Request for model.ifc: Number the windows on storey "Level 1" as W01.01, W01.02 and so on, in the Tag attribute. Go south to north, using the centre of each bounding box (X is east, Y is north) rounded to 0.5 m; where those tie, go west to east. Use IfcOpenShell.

First a look at what the model holds.

```python
import ifcopenshell
import ifcopenshell.util.element
import ifcopenshell.util.placement

model = ifcopenshell.open("model.ifc")
print(model.schema)
storey = next(s for s in model.by_type("IfcBuildingStorey") if s.Name == "Level 1")
windows = [e for e in ifcopenshell.util.element.get_decomposition(storey) if e.is_a("IfcWindow")]
for e in sorted(windows, key=lambda e: e.id()):
    origin = ifcopenshell.util.placement.get_local_placement(e.ObjectPlacement)[:3, 3]
    print(e.id(), e.Tag, e.Name, origin.round(2) + 0.0, sep=" | ")
```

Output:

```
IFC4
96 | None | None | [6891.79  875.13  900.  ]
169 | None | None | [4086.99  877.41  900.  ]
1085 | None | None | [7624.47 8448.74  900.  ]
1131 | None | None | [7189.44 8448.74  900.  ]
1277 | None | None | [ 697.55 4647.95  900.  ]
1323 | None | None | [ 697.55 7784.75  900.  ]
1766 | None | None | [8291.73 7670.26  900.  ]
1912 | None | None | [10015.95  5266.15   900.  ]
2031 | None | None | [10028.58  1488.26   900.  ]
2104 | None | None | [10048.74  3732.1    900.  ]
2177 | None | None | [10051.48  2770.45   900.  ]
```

```python
import ifcopenshell
import ifcopenshell.geom
import ifcopenshell.util.element
import ifcopenshell.util.shape

model = ifcopenshell.open("model.ifc")
settings = ifcopenshell.geom.settings()
settings.set("use-world-coords", True)


def centre(element):
    shape = ifcopenshell.geom.create_shape(settings, element)
    return ifcopenshell.util.shape.get_bbox_centroid(shape.geometry)


storey = next(s for s in model.by_type("IfcBuildingStorey") if s.Name == "Level 1")
windows = [e for e in ifcopenshell.util.element.get_decomposition(storey) if e.is_a("IfcWindow")]

# Insertion points can sit at a corner or the storey origin, so sort by the geometry (in metres).
centres = {e: centre(e) for e in windows}
windows.sort(key=lambda e: (round(centres[e][1] / 0.5), centres[e][0]))

for i, e in enumerate(windows, start=1):
    number = f"W01.{i:02d}"
    e.Tag = number
    print(e.id(), number)

model.write("model-out.ifc")
```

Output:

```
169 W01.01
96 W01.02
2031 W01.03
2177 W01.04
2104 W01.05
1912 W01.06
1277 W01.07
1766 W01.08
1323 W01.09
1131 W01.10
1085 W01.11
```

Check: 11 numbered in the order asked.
